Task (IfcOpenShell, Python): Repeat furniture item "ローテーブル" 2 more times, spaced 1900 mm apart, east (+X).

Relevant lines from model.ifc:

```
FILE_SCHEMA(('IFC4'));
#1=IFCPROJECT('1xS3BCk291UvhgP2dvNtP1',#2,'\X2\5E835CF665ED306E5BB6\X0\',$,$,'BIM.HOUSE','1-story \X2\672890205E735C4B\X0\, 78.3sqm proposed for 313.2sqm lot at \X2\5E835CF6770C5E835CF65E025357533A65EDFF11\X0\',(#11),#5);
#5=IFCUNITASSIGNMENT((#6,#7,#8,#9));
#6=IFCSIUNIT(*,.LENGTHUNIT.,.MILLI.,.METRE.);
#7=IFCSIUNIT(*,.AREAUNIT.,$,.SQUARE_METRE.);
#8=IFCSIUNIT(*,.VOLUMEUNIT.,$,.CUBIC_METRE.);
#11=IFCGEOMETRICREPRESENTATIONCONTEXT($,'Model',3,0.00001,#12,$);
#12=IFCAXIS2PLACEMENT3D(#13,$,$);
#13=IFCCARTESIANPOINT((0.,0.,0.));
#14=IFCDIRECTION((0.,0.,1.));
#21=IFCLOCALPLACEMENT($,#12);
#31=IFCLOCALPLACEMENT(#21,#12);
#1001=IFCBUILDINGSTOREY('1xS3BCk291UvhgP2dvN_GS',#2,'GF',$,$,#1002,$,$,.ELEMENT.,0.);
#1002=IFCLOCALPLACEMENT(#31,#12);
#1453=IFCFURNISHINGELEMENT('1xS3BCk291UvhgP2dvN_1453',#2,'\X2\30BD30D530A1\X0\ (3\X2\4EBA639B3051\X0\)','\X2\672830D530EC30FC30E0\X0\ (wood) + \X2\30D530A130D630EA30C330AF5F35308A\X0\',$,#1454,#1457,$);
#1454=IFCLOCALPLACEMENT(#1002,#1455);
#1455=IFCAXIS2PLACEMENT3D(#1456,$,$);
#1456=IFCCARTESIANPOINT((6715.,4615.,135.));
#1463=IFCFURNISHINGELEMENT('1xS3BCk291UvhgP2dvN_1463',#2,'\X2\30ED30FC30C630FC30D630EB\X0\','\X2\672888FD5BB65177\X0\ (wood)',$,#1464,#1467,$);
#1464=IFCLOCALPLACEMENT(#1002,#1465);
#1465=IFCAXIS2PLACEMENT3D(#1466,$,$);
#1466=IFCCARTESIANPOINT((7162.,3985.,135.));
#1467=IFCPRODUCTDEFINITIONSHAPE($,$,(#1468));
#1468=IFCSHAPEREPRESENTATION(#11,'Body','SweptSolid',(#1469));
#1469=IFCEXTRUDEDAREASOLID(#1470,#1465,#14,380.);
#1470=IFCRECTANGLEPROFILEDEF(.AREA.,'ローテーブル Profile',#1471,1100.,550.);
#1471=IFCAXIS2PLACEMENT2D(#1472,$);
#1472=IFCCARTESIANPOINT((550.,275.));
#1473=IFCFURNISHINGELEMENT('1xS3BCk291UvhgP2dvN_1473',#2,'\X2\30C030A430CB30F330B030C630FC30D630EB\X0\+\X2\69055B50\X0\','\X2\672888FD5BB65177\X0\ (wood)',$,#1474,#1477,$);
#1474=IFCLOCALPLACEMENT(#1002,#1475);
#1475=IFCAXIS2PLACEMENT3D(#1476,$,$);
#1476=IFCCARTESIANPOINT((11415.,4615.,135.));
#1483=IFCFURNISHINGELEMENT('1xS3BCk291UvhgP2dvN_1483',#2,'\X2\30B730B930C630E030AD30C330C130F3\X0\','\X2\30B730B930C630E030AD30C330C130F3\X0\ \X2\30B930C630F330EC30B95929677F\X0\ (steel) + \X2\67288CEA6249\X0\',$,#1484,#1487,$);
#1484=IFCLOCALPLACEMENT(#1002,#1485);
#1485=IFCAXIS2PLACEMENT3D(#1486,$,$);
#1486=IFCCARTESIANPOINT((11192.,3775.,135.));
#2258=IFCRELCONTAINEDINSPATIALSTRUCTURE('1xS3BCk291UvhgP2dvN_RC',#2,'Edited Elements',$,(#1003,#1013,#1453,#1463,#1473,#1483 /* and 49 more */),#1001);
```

```python
import numpy as np
import ifcopenshell
import ifcopenshell.api.geometry
import ifcopenshell.api.root
import ifcopenshell.util.element
import ifcopenshell.util.placement
import ifcopenshell.util.unit

model = ifcopenshell.open("model.ifc")
unit_scale = ifcopenshell.util.unit.calculate_unit_scale(model)


def reuse_history(source, copy):
    """copy_class also copies each property set's owner history, people and application; keep the originals."""
    for rel in copy.IsDefinedBy:
        if rel.is_a("IfcRelDefinesByProperties") and (history := rel.RelatingPropertyDefinition.OwnerHistory):
            rel.RelatingPropertyDefinition.OwnerHistory = source.OwnerHistory
            ifcopenshell.util.element.remove_deep2(model, history)


source = model.by_guid("1xS3BCk291UvhgP2dvN_1463")
base = ifcopenshell.util.placement.get_local_placement(source.ObjectPlacement)
step = np.array([1.0, 0.0, 0.0]) * 1.9 / unit_scale

for i in range(1, 3):
    copy = ifcopenshell.api.root.copy_class(model, product=source)
    copy.Representation = ifcopenshell.util.element.copy_deep(
        model, source.Representation, exclude=["IfcGeometricRepresentationContext", "IfcRepresentationMap"]
    )
    reuse_history(source, copy)
    matrix = base.copy()
    matrix[:3, 3] += i * step
    print("added at", matrix[:3, 3].round(3) + 0.0)
    ifcopenshell.api.geometry.edit_object_placement(model, product=copy, matrix=matrix, is_si=False)

model.write("model_edited.ifc")
```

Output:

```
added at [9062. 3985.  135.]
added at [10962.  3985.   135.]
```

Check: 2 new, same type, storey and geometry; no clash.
